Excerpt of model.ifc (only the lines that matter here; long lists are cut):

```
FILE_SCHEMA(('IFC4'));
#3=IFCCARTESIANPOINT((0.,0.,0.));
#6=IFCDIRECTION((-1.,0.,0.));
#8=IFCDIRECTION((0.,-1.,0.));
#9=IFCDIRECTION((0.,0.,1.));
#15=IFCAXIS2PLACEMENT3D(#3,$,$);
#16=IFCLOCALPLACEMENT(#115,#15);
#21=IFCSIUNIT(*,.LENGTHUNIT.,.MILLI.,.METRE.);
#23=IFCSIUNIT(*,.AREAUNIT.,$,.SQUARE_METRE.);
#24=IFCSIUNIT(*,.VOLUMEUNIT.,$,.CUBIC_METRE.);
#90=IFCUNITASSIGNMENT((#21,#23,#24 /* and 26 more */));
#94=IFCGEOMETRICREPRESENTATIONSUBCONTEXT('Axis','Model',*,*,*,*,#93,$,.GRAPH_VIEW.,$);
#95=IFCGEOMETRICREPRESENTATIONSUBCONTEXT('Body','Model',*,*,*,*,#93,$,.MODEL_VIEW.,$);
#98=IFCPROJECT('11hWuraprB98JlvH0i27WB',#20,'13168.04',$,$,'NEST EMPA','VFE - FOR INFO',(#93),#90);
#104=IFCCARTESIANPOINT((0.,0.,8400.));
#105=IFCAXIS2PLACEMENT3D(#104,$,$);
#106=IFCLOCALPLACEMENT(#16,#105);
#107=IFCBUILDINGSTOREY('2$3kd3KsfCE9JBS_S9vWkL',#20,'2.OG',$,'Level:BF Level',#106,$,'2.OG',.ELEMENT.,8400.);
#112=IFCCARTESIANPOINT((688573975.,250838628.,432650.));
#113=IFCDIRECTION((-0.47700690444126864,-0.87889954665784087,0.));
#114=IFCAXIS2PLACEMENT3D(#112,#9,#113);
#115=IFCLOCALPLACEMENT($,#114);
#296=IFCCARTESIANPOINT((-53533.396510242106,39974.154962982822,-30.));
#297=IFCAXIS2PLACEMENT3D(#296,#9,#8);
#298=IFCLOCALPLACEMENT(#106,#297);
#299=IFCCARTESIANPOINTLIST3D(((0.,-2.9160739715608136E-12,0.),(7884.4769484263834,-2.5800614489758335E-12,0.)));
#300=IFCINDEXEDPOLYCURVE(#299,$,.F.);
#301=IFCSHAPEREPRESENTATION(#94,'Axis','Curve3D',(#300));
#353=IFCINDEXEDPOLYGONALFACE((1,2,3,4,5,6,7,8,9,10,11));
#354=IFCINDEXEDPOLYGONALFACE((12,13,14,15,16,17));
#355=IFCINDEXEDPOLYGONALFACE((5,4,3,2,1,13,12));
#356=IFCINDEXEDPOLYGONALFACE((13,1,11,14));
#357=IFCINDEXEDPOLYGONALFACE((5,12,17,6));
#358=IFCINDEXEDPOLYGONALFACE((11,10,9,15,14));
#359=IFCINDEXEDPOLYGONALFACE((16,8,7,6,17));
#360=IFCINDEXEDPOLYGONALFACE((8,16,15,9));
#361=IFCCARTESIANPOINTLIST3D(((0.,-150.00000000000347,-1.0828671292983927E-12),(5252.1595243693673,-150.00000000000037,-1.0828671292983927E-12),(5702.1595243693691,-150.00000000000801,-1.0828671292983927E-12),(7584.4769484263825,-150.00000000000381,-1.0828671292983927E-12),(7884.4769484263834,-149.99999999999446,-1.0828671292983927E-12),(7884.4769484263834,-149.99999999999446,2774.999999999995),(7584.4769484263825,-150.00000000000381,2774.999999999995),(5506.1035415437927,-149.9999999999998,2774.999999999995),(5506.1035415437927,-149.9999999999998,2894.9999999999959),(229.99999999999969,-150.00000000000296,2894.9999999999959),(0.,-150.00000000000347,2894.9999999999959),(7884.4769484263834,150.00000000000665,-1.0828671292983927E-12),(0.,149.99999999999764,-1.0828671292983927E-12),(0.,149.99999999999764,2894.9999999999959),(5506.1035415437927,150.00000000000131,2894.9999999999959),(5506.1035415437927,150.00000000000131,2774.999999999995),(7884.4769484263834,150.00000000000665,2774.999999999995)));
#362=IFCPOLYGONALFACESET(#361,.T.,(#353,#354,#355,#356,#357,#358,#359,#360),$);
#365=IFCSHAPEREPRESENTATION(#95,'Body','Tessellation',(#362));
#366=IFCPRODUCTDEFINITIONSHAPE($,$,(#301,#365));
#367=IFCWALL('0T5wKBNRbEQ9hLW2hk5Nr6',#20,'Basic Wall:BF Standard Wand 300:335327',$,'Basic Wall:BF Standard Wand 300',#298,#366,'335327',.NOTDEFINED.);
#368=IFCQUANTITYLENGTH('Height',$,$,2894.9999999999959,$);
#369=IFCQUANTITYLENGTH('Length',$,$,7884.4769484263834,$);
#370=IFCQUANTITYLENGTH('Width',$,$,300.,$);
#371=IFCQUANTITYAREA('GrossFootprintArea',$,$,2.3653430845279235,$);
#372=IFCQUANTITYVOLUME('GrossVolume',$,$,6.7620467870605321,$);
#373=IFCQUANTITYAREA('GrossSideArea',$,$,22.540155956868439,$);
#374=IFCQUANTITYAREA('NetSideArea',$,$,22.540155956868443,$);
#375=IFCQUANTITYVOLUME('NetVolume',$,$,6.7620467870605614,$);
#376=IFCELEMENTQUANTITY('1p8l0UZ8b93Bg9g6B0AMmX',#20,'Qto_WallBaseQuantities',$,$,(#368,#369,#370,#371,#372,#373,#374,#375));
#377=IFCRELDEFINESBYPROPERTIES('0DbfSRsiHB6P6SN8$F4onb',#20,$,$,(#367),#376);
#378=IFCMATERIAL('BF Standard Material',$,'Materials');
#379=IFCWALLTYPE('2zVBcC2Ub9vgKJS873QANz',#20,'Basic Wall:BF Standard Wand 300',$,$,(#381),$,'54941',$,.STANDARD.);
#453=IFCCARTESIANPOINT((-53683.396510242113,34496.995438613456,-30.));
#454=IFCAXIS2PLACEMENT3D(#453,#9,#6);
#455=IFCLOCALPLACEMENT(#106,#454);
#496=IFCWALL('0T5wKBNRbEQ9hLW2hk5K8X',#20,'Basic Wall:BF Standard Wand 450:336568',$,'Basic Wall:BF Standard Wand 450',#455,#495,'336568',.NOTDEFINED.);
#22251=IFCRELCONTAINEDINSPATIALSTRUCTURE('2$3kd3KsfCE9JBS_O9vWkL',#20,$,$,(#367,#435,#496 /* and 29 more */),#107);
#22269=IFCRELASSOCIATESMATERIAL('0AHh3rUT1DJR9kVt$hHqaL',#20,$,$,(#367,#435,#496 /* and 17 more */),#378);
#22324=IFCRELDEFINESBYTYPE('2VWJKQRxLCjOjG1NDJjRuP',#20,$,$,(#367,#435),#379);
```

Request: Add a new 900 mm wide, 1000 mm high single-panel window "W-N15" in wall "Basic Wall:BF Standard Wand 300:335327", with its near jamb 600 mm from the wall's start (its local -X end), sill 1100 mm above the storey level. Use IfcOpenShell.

```python
import numpy as np
import ifcopenshell
import ifcopenshell.api.feature
import ifcopenshell.api.geometry
import ifcopenshell.api.pset
import ifcopenshell.api.root
import ifcopenshell.api.spatial
import ifcopenshell.geom
import ifcopenshell.util.element
import ifcopenshell.util.placement
import ifcopenshell.util.representation
import ifcopenshell.util.shape
import ifcopenshell.util.unit

model = ifcopenshell.open("model.ifc")
unit_scale = ifcopenshell.util.unit.calculate_unit_scale(model)
area_scale = ifcopenshell.util.unit.calculate_unit_scale(model, "AREAUNIT")
volume_scale = ifcopenshell.util.unit.calculate_unit_scale(model, "VOLUMEUNIT")
settings = ifcopenshell.geom.settings()


def volume(element):
    """Net volume in cubic metres, openings subtracted."""
    shape = ifcopenshell.geom.create_shape(settings, element)
    return ifcopenshell.util.shape.get_volume(shape.geometry)


wall = model.by_guid("0T5wKBNRbEQ9hLW2hk5Nr6")
storey = ifcopenshell.util.element.get_container(wall, ifc_class="IfcBuildingStorey")
context = ifcopenshell.util.representation.get_context(model, "Model", "Body", "MODEL_VIEW")
before = volume(wall)

width, height, from_end, sill = 0.9, 1, 0.6, 1.1  # metres

# The wall runs along its own X axis, and the end named is its -X end.
wall_shape = ifcopenshell.geom.create_shape(settings, wall)
x, y, z = ifcopenshell.util.shape.get_vertices(wall_shape.geometry).T
start = x.min() + from_end
face, thickness = float(y.min()), float(y.max() - y.min())
wall_matrix = ifcopenshell.util.placement.get_local_placement(wall.ObjectPlacement)
level = ifcopenshell.util.placement.get_local_placement(storey.ObjectPlacement)[2, 3]


def in_wall(x, y):
    """Placement at x, y metres in the wall's axes, at sill height."""
    matrix = wall_matrix.copy()
    matrix[:, 3] = wall_matrix @ np.array([x / unit_scale, y / unit_scale, 0.0, 1.0])
    matrix[2, 3] = level + sill / unit_scale
    return matrix


# Opening: a box that overshoots both wall faces by 50 mm.
opening = ifcopenshell.api.root.create_entity(model, ifc_class="IfcOpeningElement", predefined_type="OPENING")
box = ifcopenshell.api.geometry.add_wall_representation(
    model, context=context, length=width, height=height, thickness=thickness + 0.1
)
ifcopenshell.api.geometry.assign_representation(model, product=opening, representation=box)
ifcopenshell.api.geometry.edit_object_placement(model, product=opening, matrix=in_wall(start, face - 0.05), is_si=False)
ifcopenshell.api.feature.add_feature(model, feature=opening, element=wall)

window = ifcopenshell.api.root.create_entity(model, ifc_class="IfcWindow", name="W-N15", predefined_type="WINDOW")
window.OverallWidth, window.OverallHeight = width / unit_scale, height / unit_scale
window.PartitioningType = "SINGLE_PANEL"
body = ifcopenshell.api.geometry.add_window_representation(
    model,
    context=context,
    overall_width=window.OverallWidth,
    overall_height=window.OverallHeight,
    partition_type="SINGLE_PANEL",
)
ifcopenshell.api.geometry.assign_representation(model, product=window, representation=body)
ifcopenshell.api.spatial.assign_container(model, products=[window], relating_structure=storey)
ifcopenshell.api.feature.add_filling(model, opening=opening, element=window)

# Centre the window in the wall's thickness.
ifcopenshell.api.geometry.edit_object_placement(model, product=window, matrix=in_wall(start, face), is_si=False)
window_shape = ifcopenshell.geom.create_shape(settings, window)
depth = ifcopenshell.util.shape.get_vertices(window_shape.geometry)[:, 1]
offset = face + thickness / 2 - (depth.min() + depth.max()) / 2
ifcopenshell.api.geometry.edit_object_placement(model, product=window, matrix=in_wall(start, offset), is_si=False)

after = volume(wall)

# Update the wall's stored quantities.
qto = model.by_id(ifcopenshell.util.element.get_pset(wall, "Qto_WallBaseQuantities", should_inherit=False)["id"])
ifcopenshell.api.pset.edit_qto(model, qto=qto, properties={
    "NetSideArea": after / thickness / area_scale,
    "NetVolume": after / volume_scale,
})

print(f"wall volume {before:.3f} -> {after:.3f} m3")

model.write("model_v2.ifc")
```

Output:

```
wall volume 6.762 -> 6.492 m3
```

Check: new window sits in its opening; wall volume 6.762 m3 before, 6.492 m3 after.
